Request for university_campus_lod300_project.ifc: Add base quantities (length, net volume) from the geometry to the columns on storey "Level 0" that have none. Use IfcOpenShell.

First a look at what the model holds.

```python
import ifcopenshell
import ifcopenshell.util.element
import ifcopenshell.util.unit

model = ifcopenshell.open("university_campus_lod300_project.ifc")
print(model.schema)
for unit_type in ("LENGTHUNIT", "AREAUNIT", "VOLUMEUNIT"):
    print(unit_type, ifcopenshell.util.unit.calculate_unit_scale(model, unit_type))
storey = next(s for s in model.by_type("IfcBuildingStorey") if s.Name == "Level 0")
columns = [e for e in ifcopenshell.util.element.get_decomposition(storey) if e.is_a("IfcColumn")]
for e in sorted(columns, key=lambda e: e.id()):
    print(e.id(), e.is_a(), e.Name, list(ifcopenshell.util.element.get_psets(e, qtos_only=True)), sep=" | ")
```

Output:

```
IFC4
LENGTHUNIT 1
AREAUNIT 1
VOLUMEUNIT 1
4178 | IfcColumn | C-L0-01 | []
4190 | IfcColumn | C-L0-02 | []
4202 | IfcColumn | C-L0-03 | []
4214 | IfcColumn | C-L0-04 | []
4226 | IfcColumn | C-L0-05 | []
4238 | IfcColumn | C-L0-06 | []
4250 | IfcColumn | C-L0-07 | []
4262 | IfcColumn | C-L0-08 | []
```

```python
import ifcopenshell
import ifcopenshell.api.pset
import ifcopenshell.geom
import ifcopenshell.util.element
import ifcopenshell.util.shape
import ifcopenshell.util.unit

model = ifcopenshell.open("university_campus_lod300_project.ifc")
unit_scale = ifcopenshell.util.unit.calculate_unit_scale(model)
volume_scale = ifcopenshell.util.unit.calculate_unit_scale(model, "VOLUMEUNIT")
settings = ifcopenshell.geom.settings()

storey = next(s for s in model.by_type("IfcBuildingStorey") if s.Name == "Level 0")
columns = [e for e in ifcopenshell.util.element.get_decomposition(storey) if e.is_a("IfcColumn")]

for e in sorted(columns, key=lambda e: e.id()):
    if ifcopenshell.util.element.get_psets(e, qtos_only=True, should_inherit=False):
        continue
    # Geometry comes back in metres, in the element's own axes.
    shape = ifcopenshell.geom.create_shape(settings, e)
    values = {
        "Length": ifcopenshell.util.shape.get_z(shape.geometry) / unit_scale,
        "NetVolume": ifcopenshell.util.shape.get_volume(shape.geometry) / volume_scale,
    }
    qto = ifcopenshell.api.pset.add_qto(model, product=e, name="Qto_ColumnBaseQuantities")
    ifcopenshell.api.pset.edit_qto(model, qto=qto, properties=values)
    print(e.id(), {k: round(v, 3) for k, v in values.items()})

model.write("university_campus_lod300_project-out.ifc")
```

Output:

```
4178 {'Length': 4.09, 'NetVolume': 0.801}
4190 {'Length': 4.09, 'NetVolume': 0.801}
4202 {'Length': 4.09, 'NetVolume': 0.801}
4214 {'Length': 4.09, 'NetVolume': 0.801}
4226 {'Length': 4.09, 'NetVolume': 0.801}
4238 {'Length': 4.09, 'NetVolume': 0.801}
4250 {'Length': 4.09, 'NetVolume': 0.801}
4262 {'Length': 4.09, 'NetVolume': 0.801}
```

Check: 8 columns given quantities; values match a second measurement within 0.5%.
